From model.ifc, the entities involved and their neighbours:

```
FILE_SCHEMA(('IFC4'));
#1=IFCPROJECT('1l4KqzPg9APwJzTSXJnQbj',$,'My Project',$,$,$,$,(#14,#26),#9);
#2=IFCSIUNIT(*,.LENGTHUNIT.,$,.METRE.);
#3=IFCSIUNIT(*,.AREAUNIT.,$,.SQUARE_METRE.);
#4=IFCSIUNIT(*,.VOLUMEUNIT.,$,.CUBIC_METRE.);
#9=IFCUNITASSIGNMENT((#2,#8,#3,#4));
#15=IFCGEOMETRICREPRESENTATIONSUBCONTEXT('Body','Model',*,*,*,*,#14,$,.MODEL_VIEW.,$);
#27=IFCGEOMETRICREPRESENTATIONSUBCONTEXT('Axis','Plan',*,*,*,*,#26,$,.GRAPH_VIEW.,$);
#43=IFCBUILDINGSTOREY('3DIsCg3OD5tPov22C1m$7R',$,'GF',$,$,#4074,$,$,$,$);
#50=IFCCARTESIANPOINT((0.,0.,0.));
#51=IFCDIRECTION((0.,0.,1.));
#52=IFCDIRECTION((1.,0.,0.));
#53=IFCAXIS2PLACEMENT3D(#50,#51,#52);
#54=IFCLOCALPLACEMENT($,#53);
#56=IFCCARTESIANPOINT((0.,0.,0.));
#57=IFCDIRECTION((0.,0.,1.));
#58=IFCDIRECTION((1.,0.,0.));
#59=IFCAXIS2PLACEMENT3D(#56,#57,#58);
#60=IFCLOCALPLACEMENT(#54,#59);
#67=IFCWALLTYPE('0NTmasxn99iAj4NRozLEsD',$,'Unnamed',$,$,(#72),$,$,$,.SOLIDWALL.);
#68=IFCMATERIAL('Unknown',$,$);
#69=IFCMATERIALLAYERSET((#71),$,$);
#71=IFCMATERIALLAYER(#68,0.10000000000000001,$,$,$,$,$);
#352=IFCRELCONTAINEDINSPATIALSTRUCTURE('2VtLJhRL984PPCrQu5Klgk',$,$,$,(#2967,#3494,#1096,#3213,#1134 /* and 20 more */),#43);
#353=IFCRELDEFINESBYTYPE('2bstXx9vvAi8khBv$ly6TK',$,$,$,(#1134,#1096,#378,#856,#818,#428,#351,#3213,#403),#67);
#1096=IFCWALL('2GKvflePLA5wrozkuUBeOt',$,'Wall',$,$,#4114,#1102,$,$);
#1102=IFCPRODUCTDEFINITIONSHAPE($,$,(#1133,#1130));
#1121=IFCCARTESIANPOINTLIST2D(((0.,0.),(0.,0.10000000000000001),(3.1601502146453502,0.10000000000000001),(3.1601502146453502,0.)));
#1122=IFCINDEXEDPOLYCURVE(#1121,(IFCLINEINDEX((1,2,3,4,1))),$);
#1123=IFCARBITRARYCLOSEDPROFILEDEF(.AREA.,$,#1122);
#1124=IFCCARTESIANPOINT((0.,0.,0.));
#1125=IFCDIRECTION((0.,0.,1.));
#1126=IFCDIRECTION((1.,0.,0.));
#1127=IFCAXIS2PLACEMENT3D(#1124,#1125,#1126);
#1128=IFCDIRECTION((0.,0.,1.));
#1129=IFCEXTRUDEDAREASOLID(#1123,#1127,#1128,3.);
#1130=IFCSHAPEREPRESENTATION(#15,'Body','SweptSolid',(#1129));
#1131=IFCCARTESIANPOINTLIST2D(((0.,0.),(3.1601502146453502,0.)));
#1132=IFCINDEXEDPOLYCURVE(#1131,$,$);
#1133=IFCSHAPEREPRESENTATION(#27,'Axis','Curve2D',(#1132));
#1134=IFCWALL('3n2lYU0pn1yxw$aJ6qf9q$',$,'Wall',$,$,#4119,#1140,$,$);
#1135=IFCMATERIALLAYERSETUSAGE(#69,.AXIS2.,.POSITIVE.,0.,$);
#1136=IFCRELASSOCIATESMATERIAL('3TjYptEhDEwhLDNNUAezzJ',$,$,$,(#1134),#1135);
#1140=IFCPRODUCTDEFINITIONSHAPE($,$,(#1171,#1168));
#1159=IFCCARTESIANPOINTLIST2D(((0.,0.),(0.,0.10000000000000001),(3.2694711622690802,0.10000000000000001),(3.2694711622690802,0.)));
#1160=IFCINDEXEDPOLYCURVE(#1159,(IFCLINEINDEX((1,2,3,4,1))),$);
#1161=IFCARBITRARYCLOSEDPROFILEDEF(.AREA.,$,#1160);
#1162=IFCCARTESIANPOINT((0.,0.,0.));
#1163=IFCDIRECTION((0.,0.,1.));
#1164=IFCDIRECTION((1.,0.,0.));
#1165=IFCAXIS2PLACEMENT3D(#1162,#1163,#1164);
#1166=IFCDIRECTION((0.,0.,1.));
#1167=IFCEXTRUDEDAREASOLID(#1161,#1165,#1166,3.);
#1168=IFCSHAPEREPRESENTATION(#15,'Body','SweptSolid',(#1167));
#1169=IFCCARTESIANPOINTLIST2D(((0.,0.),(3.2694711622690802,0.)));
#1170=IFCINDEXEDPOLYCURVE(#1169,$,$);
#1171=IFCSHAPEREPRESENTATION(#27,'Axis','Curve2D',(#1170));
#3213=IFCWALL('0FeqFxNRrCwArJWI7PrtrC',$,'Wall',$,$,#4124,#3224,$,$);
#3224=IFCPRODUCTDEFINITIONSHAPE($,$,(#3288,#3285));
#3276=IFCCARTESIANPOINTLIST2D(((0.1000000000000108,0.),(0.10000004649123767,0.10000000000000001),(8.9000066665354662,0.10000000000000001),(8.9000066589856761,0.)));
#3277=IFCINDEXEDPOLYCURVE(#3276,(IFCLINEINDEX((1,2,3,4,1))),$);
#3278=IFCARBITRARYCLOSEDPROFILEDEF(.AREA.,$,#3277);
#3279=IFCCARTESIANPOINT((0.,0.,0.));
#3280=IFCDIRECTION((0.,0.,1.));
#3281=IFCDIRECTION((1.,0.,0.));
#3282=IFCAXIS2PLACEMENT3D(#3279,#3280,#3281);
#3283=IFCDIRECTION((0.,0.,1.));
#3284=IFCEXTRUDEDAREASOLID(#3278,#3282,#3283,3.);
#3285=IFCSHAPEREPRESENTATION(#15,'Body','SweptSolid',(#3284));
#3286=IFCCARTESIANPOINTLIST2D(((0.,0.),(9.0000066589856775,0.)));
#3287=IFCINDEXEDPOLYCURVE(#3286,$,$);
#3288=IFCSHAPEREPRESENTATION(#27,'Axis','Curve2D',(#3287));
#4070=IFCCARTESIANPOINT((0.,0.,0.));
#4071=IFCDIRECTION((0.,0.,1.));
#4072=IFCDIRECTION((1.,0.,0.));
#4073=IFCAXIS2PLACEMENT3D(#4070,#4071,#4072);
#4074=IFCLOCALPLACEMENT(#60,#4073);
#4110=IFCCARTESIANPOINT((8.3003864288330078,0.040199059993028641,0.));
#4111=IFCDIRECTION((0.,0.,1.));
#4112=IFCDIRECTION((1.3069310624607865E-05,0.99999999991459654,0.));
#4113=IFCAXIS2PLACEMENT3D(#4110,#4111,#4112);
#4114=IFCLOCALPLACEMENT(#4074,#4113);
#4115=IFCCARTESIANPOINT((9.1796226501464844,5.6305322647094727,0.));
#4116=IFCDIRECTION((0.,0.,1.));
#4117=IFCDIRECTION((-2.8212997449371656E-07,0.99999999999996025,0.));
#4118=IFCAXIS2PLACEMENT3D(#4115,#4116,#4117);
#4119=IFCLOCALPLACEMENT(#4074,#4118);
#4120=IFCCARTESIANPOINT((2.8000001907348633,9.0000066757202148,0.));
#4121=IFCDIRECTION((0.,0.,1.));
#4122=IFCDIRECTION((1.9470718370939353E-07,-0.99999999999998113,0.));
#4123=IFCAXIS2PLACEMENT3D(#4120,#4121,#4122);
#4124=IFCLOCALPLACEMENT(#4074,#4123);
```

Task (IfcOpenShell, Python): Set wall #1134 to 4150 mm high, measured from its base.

```python
import ifcopenshell
import ifcopenshell.geom
import ifcopenshell.util.representation
import ifcopenshell.util.shape
import ifcopenshell.util.unit

model = ifcopenshell.open("model.ifc")
unit_scale = ifcopenshell.util.unit.calculate_unit_scale(model)
settings = ifcopenshell.geom.settings()


def volume(element):
    """Net volume in cubic metres, openings subtracted."""
    shape = ifcopenshell.geom.create_shape(settings, element)
    return ifcopenshell.util.shape.get_volume(shape.geometry)


wall = model.by_id(1134)
before = volume(wall)

body = ifcopenshell.util.representation.get_representation(wall, "Model", "Body")
solid = body.Items[0]
old_height = solid.Depth
solid.Depth = 4.15 / unit_scale
after = volume(wall)

print(f"height {old_height:g} -> {solid.Depth:g}, volume {before:.3f} -> {after:.3f} m3")

model.write("model_updated.ifc")
```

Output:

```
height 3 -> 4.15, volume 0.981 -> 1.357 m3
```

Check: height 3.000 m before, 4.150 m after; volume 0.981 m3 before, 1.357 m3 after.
